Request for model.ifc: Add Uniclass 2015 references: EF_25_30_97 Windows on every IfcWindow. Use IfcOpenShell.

First a look at what the model holds.

```python
import ifcopenshell

model = ifcopenshell.open("model.ifc")
print(model.schema)
print("classifications:", [c.Name for c in model.by_type("IfcClassification")])
for ifc_class in ("IfcDoor", "IfcRoof", "IfcStair", "IfcWall", "IfcWindow"):
    print(ifc_class, len(model.by_type(ifc_class)))
```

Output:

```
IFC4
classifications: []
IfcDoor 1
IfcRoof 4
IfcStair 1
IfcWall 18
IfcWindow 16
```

```python
import ifcopenshell
import ifcopenshell.api.classification

model = ifcopenshell.open("model.ifc")

system = ifcopenshell.api.classification.add_classification(model, classification="Uniclass 2015")

codes = {
    "IfcWindow": ("EF_25_30_97", "Windows"),
}
for ifc_class, (code, name) in codes.items():
    products = model.by_type(ifc_class)
    ifcopenshell.api.classification.add_reference(
        model, products=products, classification=system, identification=code, name=name
    )
    print(code, len(products))

model.write("model-out.ifc")
```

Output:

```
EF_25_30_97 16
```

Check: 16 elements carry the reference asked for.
